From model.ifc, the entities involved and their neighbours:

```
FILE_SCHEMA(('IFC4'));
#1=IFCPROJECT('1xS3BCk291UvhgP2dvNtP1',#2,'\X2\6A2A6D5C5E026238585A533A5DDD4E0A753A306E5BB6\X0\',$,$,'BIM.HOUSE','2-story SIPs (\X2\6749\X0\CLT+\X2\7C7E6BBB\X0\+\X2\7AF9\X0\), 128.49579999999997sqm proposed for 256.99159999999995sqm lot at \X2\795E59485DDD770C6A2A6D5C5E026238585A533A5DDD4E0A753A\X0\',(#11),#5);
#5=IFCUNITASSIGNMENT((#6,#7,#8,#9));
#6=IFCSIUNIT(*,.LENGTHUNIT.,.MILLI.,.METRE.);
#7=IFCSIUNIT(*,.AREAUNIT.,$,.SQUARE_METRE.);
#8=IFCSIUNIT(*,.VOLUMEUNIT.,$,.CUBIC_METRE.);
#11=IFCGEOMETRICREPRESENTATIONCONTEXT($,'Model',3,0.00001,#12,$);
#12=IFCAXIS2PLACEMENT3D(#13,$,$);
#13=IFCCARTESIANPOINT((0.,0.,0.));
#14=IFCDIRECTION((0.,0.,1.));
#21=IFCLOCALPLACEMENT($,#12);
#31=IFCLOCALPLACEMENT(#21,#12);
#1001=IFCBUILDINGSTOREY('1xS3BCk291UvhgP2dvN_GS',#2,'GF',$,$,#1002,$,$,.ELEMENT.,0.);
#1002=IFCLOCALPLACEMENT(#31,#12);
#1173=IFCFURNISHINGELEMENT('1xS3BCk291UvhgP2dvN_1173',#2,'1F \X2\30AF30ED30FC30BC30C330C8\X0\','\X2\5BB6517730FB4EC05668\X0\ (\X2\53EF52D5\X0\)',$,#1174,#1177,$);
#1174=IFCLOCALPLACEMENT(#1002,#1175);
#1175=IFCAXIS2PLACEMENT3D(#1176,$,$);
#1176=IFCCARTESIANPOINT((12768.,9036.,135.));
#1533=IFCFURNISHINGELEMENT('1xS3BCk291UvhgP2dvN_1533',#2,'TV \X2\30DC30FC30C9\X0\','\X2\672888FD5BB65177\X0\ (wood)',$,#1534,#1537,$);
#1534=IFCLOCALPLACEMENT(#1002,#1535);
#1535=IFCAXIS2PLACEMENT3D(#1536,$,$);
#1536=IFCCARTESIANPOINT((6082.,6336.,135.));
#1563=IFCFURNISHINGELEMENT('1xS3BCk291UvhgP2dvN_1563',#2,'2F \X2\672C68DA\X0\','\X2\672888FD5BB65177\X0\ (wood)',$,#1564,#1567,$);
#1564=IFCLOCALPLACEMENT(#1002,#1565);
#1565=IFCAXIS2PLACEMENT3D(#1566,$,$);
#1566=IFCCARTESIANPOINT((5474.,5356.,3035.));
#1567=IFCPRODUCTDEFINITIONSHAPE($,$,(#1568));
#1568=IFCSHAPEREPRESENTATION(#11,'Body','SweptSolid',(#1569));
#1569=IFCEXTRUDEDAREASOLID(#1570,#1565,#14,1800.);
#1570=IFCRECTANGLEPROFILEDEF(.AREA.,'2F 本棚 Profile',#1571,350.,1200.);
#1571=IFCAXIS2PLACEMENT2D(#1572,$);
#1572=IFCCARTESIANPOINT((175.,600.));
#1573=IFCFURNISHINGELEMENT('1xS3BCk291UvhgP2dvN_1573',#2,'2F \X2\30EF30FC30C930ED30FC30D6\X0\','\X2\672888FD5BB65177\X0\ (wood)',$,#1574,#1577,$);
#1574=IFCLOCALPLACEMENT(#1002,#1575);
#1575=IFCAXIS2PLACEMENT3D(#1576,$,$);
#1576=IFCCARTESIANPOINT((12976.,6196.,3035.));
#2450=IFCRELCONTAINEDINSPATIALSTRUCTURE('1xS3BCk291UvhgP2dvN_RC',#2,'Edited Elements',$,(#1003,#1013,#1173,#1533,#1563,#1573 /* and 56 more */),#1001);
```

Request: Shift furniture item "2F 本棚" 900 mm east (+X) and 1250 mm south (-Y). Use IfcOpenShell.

```python
import ifcopenshell
import ifcopenshell.api.geometry
import ifcopenshell.util.placement

model = ifcopenshell.open("model.ifc")

item = model.by_guid("1xS3BCk291UvhgP2dvN_1563")
matrix = ifcopenshell.util.placement.get_local_placement(item.ObjectPlacement)
matrix[0, 3] += 900.0
matrix[1, 3] -= 1250.0
ifcopenshell.api.geometry.edit_object_placement(model, product=item, matrix=matrix, is_si=False)

print(ifcopenshell.util.placement.get_local_placement(item.ObjectPlacement).round(3) + 0.0)

model.write("model_updated.ifc")
```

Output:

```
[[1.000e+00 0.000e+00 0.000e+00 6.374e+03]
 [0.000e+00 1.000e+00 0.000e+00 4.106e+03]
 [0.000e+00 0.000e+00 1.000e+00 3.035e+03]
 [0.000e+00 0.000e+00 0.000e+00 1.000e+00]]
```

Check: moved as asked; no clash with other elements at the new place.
